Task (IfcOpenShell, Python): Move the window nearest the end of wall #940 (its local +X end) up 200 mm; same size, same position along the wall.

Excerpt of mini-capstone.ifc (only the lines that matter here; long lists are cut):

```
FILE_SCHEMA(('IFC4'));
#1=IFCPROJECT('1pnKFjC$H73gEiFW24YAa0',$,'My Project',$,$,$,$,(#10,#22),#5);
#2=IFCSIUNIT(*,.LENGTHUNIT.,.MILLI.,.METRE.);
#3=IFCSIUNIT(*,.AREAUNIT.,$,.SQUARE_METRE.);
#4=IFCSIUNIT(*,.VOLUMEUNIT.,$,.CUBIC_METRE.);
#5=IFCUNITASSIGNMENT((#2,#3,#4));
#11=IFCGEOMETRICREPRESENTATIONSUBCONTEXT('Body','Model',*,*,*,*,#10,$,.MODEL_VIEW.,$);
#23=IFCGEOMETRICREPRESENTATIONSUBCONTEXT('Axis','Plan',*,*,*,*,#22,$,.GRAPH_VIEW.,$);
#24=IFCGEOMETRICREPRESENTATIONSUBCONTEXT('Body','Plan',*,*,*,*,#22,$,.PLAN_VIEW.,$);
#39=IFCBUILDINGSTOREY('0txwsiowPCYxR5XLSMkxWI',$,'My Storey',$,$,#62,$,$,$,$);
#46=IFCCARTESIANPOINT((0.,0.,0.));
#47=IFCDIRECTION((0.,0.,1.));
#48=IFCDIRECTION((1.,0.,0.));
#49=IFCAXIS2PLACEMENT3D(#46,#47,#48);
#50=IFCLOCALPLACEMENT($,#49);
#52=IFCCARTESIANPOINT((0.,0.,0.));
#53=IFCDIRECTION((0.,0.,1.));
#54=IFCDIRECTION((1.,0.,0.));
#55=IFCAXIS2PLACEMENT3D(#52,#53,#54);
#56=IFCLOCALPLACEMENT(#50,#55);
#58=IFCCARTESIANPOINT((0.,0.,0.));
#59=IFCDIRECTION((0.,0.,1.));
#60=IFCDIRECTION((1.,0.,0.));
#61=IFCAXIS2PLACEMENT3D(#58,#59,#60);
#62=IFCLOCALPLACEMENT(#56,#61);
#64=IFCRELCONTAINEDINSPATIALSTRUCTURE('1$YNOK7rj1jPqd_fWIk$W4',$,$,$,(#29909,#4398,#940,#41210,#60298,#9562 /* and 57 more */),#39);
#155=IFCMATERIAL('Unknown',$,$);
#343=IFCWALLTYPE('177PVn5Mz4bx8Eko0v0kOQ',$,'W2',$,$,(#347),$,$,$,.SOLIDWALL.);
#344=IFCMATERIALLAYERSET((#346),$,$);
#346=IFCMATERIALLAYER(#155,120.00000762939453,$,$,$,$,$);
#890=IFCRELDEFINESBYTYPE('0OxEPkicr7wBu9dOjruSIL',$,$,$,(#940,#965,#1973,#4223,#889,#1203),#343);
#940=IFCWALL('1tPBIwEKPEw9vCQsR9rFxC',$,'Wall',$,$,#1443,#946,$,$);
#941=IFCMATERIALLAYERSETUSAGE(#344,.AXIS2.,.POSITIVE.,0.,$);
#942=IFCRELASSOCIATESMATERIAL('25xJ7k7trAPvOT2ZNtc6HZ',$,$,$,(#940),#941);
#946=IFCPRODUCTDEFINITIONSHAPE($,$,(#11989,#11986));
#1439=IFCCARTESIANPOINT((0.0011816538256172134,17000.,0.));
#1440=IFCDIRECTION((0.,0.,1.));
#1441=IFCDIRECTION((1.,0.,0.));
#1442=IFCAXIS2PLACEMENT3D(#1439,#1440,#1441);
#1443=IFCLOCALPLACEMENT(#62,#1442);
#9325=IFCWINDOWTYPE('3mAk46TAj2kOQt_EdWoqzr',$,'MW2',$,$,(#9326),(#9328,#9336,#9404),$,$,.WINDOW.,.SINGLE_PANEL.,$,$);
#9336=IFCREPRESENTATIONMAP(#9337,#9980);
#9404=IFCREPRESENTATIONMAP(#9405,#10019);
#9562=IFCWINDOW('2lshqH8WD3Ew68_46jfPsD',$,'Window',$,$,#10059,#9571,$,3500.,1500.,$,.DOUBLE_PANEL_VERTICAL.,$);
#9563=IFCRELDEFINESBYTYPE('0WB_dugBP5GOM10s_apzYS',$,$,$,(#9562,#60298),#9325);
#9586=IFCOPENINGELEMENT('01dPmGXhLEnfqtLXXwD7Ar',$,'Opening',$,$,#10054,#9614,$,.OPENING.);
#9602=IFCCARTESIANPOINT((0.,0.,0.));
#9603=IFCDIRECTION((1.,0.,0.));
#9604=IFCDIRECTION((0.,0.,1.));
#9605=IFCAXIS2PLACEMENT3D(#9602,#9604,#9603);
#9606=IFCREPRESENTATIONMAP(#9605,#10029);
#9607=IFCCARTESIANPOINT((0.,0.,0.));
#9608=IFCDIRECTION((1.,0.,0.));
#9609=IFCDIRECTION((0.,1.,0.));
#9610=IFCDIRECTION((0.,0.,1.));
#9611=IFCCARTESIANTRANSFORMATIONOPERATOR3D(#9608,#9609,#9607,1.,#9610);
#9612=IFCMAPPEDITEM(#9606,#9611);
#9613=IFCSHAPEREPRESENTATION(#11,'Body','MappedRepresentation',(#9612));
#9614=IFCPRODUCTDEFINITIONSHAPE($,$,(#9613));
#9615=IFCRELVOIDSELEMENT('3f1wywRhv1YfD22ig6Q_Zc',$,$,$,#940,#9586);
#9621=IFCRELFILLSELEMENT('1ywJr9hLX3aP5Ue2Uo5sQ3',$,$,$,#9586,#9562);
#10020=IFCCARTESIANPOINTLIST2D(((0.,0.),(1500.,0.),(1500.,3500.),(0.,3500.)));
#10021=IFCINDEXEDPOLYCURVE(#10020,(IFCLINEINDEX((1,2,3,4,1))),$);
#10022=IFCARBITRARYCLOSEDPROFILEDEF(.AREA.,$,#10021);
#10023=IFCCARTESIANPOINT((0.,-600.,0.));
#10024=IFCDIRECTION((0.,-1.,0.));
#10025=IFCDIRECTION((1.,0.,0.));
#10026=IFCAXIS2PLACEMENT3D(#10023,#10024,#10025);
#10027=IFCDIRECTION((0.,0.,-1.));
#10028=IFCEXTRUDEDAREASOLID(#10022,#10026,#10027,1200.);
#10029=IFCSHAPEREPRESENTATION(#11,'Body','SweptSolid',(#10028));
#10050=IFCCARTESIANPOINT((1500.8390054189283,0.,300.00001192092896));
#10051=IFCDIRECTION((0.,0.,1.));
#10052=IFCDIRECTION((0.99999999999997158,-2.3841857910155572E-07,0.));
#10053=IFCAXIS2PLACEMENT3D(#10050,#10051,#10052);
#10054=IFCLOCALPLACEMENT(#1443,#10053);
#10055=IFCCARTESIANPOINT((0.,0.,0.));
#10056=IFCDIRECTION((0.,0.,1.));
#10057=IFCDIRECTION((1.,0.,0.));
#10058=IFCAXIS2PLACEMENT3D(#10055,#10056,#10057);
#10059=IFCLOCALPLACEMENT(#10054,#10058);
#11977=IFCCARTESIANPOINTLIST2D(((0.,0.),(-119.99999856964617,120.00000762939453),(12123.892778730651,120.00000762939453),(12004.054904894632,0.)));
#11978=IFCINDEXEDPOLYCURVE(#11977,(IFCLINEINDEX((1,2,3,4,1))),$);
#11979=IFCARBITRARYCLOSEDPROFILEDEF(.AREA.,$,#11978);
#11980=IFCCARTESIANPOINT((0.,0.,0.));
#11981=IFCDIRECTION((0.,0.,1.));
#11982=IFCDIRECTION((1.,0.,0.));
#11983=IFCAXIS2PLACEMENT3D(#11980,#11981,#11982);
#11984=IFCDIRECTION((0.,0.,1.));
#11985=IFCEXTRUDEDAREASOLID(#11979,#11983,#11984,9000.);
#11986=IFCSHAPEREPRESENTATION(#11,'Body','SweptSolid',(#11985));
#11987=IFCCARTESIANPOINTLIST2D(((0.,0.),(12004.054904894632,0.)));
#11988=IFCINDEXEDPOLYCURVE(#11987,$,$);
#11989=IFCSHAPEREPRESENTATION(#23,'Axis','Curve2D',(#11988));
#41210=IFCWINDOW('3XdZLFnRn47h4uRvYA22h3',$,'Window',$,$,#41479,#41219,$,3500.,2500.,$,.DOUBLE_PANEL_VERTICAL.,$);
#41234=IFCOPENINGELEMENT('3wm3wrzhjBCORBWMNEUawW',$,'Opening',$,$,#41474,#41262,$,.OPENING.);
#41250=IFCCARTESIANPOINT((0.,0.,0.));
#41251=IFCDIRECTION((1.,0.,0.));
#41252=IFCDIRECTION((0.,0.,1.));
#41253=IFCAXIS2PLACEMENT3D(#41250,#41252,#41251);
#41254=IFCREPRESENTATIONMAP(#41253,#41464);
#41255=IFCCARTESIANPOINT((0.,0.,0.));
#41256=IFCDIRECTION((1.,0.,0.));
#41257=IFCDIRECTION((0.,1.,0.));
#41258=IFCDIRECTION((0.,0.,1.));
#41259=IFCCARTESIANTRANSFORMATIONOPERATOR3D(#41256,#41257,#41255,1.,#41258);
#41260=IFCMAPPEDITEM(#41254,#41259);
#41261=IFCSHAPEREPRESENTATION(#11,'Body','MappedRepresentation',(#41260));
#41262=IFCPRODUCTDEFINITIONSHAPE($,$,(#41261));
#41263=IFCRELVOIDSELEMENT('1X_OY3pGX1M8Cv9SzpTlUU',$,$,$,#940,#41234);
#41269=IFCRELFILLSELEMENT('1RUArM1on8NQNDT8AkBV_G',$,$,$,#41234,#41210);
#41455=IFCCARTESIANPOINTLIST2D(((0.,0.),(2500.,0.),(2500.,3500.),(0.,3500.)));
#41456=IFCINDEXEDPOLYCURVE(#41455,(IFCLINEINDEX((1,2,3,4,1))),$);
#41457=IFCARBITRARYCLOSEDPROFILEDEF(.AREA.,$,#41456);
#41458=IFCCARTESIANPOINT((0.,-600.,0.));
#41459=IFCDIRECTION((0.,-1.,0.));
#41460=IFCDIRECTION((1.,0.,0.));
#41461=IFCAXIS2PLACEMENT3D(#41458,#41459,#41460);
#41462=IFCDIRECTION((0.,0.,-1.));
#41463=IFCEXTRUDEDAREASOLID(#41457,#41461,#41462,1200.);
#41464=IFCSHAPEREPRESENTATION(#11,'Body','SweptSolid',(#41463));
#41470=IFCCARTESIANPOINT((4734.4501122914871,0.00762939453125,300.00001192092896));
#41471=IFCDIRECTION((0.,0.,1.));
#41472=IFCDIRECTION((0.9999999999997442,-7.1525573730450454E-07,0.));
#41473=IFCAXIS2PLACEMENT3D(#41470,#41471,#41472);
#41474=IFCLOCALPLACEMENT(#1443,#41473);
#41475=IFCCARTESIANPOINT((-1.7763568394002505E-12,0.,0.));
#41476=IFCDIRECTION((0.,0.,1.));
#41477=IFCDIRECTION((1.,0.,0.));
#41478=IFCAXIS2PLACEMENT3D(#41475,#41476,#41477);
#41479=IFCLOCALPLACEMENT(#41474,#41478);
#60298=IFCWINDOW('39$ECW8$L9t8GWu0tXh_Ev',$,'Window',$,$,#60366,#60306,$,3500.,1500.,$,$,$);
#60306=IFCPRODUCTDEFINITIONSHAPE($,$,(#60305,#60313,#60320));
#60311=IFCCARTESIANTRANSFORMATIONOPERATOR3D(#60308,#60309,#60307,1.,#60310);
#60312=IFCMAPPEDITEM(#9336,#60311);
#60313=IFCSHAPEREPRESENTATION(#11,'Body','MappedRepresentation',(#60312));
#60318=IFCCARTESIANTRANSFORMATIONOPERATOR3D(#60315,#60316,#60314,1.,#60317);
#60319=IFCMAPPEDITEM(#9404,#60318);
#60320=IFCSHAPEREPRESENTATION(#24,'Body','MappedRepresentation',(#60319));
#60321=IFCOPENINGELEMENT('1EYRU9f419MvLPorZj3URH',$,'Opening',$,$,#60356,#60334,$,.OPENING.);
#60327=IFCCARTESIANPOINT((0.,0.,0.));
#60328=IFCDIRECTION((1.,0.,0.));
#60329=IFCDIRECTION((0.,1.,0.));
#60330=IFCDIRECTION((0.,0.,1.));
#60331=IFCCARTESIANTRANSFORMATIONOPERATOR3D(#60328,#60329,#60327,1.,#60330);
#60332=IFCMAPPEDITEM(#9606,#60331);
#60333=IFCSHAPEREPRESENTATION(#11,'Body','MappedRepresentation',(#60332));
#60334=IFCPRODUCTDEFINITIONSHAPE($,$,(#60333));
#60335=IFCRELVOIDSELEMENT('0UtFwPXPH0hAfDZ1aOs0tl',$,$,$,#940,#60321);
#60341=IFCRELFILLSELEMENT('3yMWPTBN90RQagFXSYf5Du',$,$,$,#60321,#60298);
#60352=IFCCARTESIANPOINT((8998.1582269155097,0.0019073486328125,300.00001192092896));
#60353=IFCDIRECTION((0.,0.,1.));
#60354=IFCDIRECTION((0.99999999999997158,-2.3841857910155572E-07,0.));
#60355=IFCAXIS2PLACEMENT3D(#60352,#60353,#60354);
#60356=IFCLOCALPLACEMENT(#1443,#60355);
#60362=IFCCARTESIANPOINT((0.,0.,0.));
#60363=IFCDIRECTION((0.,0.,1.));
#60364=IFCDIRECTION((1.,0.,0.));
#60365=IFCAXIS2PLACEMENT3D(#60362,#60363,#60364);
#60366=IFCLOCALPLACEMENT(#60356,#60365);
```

```python
import numpy as np
import ifcopenshell
import ifcopenshell.api.geometry
import ifcopenshell.util.placement
import ifcopenshell.util.unit

model = ifcopenshell.open("mini-capstone.ifc")
unit_scale = ifcopenshell.util.unit.calculate_unit_scale(model)

window = model.by_id(60298)
opening = window.FillsVoids[0].RelatingOpeningElement
dz = 0.2 / unit_scale

shift = np.array([0.0, 0.0, dz])
# The window is placed relative to its opening, so it follows when the opening moves.
matrix = ifcopenshell.util.placement.get_local_placement(opening.ObjectPlacement)
matrix[:3, 3] += shift
ifcopenshell.api.geometry.edit_object_placement(
    model, product=opening, matrix=matrix, is_si=False, should_transform_children=True
)

print(f"moved by {dz * unit_scale:+.3f} m")

model.write("mini-capstone_rev.ifc")
```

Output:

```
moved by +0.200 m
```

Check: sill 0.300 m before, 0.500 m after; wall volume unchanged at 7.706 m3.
